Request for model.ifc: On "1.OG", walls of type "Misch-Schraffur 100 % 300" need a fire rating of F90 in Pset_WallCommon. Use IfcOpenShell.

First a look at what the model holds.

```python
import ifcopenshell
import ifcopenshell.util.element

model = ifcopenshell.open("model.ifc")
print(model.schema)
storey = next(s for s in model.by_type("IfcBuildingStorey") if s.Name == "1.OG")
walls = [e for e in ifcopenshell.util.element.get_decomposition(storey) if e.is_a("IfcWall")]
seen = {}
for e in walls:
    element_type = ifcopenshell.util.element.get_type(e)
    key = (element_type.Name if element_type != e and element_type else None, ifcopenshell.util.element.get_pset(e, "Pset_WallCommon", "FireRating"))
    seen[key] = seen.get(key, 0) + 1
for (name, value), count in sorted(seen.items(), key=str):
    print(count, "x", name, "|", value)
```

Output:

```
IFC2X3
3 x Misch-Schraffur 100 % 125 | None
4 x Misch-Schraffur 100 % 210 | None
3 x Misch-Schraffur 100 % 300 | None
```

```python
import ifcopenshell
import ifcopenshell.api.pset
import ifcopenshell.util.element

model = ifcopenshell.open("model.ifc")

storey = next(s for s in model.by_type("IfcBuildingStorey") if s.Name == "1.OG")
walls = [e for e in ifcopenshell.util.element.get_decomposition(storey) if e.is_a("IfcWall")]

count = 0
for e in walls:
    element_type = ifcopenshell.util.element.get_type(e)
    if element_type in (None, e) or element_type.Name != "Misch-Schraffur 100 % 300":
        continue
    # add_pset returns the element's existing set when there is one.
    pset = ifcopenshell.api.pset.add_pset(model, product=e, name="Pset_WallCommon")
    ifcopenshell.api.pset.edit_pset(model, pset=pset, properties={"FireRating": "F90"})
    count += 1

print(count, "walls updated")

model.write("model_v2.ifc")
```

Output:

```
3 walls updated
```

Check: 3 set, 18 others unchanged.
